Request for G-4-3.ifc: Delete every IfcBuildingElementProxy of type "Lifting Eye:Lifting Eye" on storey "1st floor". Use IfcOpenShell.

First a look at what the model holds.

```python
import ifcopenshell
import ifcopenshell.util.element

model = ifcopenshell.open("G-4-3.ifc")
print(model.schema)
storey = next(s for s in model.by_type("IfcBuildingStorey") if s.Name == "1st floor")
proxies = [e for e in ifcopenshell.util.element.get_decomposition(storey) if e.is_a("IfcBuildingElementProxy")]
seen = {}
for e in proxies:
    element_type = ifcopenshell.util.element.get_type(e)
    name = element_type.Name if element_type not in (None, e) else None
    seen[name] = seen.get(name, 0) + 1
for name, count in sorted(seen.items(), key=str):
    print(count, "x", name)
```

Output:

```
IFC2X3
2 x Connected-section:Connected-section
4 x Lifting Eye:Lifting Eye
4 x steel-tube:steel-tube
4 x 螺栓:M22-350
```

```python
import ifcopenshell
import ifcopenshell.api.root
import ifcopenshell.util.element

model = ifcopenshell.open("G-4-3.ifc")

storey = next(s for s in model.by_type("IfcBuildingStorey") if s.Name == "1st floor")
proxies = [e for e in ifcopenshell.util.element.get_decomposition(storey) if e.is_a("IfcBuildingElementProxy")]
targets = [e for e in proxies if (t := ifcopenshell.util.element.get_type(e)) not in (None, e) and t.Name == "Lifting Eye:Lifting Eye"]

for e in targets:
    ifcopenshell.api.root.remove_product(model, product=e)
print(len(targets), "removed")

model.write("G-4-3_updated.ifc")
```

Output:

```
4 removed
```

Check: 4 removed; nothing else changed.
